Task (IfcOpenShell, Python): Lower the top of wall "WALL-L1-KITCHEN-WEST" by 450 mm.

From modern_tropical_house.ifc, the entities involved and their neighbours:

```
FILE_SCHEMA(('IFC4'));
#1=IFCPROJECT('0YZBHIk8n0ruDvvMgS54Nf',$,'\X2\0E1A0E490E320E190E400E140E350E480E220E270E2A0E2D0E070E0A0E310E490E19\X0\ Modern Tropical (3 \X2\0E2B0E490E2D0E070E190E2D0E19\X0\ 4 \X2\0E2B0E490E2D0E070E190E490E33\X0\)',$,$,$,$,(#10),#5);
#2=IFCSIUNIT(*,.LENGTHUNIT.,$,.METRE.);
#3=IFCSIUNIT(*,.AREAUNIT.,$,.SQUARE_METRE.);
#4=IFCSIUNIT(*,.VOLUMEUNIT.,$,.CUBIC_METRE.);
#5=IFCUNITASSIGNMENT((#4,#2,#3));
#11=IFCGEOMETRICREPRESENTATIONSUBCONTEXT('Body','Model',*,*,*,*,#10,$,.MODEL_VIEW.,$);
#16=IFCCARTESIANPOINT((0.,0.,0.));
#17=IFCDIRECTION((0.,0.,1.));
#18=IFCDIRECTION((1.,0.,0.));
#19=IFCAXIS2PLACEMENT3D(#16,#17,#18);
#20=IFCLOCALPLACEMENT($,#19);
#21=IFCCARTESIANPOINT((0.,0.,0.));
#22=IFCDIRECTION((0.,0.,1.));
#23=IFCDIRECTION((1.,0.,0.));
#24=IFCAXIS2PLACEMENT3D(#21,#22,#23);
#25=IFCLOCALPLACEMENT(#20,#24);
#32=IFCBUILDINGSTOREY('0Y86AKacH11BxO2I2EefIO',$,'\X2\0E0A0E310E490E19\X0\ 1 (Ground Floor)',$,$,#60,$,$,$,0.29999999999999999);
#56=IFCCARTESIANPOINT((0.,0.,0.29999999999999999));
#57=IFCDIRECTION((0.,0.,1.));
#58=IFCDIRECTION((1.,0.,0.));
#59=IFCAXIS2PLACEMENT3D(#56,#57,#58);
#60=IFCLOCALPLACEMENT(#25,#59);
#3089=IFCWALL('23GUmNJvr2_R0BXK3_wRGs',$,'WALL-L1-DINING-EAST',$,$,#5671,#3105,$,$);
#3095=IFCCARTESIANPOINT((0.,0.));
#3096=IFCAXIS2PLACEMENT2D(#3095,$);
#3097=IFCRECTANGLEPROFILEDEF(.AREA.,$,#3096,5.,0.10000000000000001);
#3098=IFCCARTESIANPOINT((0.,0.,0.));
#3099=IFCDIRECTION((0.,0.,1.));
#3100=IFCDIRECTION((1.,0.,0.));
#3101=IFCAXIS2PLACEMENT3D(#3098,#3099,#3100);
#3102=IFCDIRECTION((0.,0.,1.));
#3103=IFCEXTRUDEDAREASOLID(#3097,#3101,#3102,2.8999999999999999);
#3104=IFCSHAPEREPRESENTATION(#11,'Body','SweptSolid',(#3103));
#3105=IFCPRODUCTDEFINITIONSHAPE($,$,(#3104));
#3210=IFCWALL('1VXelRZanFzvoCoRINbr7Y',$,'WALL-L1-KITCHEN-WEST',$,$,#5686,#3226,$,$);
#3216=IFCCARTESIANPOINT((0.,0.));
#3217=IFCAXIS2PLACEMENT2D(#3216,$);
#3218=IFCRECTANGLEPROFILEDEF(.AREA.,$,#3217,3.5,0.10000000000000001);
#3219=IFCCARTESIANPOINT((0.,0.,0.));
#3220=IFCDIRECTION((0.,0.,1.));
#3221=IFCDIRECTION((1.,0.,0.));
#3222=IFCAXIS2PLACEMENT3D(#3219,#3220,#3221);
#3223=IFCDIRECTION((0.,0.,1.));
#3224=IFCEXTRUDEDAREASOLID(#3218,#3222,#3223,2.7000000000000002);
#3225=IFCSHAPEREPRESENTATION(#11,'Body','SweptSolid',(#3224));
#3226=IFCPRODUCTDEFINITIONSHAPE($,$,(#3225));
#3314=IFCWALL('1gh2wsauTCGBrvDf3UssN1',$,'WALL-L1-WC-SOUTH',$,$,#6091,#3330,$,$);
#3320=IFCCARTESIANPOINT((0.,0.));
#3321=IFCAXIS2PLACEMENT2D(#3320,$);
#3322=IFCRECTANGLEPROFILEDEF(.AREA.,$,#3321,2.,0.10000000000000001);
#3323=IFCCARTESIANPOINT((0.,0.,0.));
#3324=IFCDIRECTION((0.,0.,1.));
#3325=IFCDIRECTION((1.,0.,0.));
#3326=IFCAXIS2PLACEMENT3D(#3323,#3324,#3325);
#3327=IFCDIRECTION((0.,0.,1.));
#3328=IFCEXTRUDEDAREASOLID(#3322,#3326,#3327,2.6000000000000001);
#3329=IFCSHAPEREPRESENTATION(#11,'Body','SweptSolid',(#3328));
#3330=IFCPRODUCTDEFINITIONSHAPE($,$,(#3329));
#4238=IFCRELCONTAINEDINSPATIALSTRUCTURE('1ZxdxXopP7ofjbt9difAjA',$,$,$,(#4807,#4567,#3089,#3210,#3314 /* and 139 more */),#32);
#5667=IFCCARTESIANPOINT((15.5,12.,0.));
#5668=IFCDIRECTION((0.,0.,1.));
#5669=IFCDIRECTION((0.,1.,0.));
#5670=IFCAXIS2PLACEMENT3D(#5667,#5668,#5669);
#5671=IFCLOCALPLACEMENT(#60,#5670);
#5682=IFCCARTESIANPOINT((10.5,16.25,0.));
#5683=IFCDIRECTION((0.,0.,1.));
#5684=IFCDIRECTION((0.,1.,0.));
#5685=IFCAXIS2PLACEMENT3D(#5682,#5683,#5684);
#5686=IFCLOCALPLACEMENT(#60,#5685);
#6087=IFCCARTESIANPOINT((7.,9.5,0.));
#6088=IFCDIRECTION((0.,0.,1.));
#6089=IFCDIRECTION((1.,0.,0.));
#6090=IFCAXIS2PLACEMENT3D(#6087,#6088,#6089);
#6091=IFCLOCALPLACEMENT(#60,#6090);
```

```python
import ifcopenshell
import ifcopenshell.geom
import ifcopenshell.util.representation
import ifcopenshell.util.shape

model = ifcopenshell.open("modern_tropical_house.ifc")
settings = ifcopenshell.geom.settings()


def volume(element):
    """Net volume in cubic metres, openings subtracted."""
    shape = ifcopenshell.geom.create_shape(settings, element)
    return ifcopenshell.util.shape.get_volume(shape.geometry)


wall = model.by_guid("1VXelRZanFzvoCoRINbr7Y")
before = volume(wall)

body = ifcopenshell.util.representation.get_representation(wall, "Model", "Body")
solid = body.Items[0]
old_height = solid.Depth
solid.Depth -= 0.45
after = volume(wall)

print(f"height {old_height:g} -> {solid.Depth:g}, volume {before:.3f} -> {after:.3f} m3")

model.write("modern_tropical_house_rev.ifc")
```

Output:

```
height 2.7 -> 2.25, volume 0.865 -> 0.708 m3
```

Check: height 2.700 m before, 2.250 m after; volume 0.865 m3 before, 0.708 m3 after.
